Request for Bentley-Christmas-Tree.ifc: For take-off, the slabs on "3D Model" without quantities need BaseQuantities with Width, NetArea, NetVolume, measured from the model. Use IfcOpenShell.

First a look at what the model holds.

```python
import ifcopenshell
import ifcopenshell.util.element
import ifcopenshell.util.unit

model = ifcopenshell.open("Bentley-Christmas-Tree.ifc")
print(model.schema)
for unit_type in ("LENGTHUNIT", "AREAUNIT", "VOLUMEUNIT"):
    print(unit_type, ifcopenshell.util.unit.calculate_unit_scale(model, unit_type))
storey = next(s for s in model.by_type("IfcBuildingStorey") if s.Name == "3D Model")
slabs = [e for e in ifcopenshell.util.element.get_decomposition(storey) if e.is_a("IfcSlab")]
for e in sorted(slabs, key=lambda e: e.id()):
    print(e.id(), e.is_a(), e.Name, list(ifcopenshell.util.element.get_psets(e, qtos_only=True)), sep=" | ")
```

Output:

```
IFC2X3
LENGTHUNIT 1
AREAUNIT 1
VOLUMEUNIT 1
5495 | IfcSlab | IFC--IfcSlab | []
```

```python
import ifcopenshell
import ifcopenshell.api.pset
import ifcopenshell.geom
import ifcopenshell.util.element
import ifcopenshell.util.shape
import ifcopenshell.util.unit

model = ifcopenshell.open("Bentley-Christmas-Tree.ifc")
unit_scale = ifcopenshell.util.unit.calculate_unit_scale(model)
area_scale = ifcopenshell.util.unit.calculate_unit_scale(model, "AREAUNIT")
volume_scale = ifcopenshell.util.unit.calculate_unit_scale(model, "VOLUMEUNIT")
settings = ifcopenshell.geom.settings()

storey = next(s for s in model.by_type("IfcBuildingStorey") if s.Name == "3D Model")
slabs = [e for e in ifcopenshell.util.element.get_decomposition(storey) if e.is_a("IfcSlab")]

for e in sorted(slabs, key=lambda e: e.id()):
    if ifcopenshell.util.element.get_psets(e, qtos_only=True, should_inherit=False):
        continue
    # Geometry comes back in metres, in the element's own axes.
    shape = ifcopenshell.geom.create_shape(settings, e)
    values = {
        "Width": ifcopenshell.util.shape.get_z(shape.geometry) / unit_scale,
        "NetArea": ifcopenshell.util.shape.get_footprint_area(shape.geometry) / area_scale,
        "NetVolume": ifcopenshell.util.shape.get_volume(shape.geometry) / volume_scale,
    }
    qto = ifcopenshell.api.pset.add_qto(model, product=e, name="BaseQuantities")
    ifcopenshell.api.pset.edit_qto(model, qto=qto, properties=values)
    print(e.id(), {k: round(v, 3) for k, v in values.items()})

model.write("Bentley-Christmas-Tree_v2.ifc")
```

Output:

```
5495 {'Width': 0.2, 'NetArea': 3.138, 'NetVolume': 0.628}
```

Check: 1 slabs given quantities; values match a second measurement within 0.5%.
